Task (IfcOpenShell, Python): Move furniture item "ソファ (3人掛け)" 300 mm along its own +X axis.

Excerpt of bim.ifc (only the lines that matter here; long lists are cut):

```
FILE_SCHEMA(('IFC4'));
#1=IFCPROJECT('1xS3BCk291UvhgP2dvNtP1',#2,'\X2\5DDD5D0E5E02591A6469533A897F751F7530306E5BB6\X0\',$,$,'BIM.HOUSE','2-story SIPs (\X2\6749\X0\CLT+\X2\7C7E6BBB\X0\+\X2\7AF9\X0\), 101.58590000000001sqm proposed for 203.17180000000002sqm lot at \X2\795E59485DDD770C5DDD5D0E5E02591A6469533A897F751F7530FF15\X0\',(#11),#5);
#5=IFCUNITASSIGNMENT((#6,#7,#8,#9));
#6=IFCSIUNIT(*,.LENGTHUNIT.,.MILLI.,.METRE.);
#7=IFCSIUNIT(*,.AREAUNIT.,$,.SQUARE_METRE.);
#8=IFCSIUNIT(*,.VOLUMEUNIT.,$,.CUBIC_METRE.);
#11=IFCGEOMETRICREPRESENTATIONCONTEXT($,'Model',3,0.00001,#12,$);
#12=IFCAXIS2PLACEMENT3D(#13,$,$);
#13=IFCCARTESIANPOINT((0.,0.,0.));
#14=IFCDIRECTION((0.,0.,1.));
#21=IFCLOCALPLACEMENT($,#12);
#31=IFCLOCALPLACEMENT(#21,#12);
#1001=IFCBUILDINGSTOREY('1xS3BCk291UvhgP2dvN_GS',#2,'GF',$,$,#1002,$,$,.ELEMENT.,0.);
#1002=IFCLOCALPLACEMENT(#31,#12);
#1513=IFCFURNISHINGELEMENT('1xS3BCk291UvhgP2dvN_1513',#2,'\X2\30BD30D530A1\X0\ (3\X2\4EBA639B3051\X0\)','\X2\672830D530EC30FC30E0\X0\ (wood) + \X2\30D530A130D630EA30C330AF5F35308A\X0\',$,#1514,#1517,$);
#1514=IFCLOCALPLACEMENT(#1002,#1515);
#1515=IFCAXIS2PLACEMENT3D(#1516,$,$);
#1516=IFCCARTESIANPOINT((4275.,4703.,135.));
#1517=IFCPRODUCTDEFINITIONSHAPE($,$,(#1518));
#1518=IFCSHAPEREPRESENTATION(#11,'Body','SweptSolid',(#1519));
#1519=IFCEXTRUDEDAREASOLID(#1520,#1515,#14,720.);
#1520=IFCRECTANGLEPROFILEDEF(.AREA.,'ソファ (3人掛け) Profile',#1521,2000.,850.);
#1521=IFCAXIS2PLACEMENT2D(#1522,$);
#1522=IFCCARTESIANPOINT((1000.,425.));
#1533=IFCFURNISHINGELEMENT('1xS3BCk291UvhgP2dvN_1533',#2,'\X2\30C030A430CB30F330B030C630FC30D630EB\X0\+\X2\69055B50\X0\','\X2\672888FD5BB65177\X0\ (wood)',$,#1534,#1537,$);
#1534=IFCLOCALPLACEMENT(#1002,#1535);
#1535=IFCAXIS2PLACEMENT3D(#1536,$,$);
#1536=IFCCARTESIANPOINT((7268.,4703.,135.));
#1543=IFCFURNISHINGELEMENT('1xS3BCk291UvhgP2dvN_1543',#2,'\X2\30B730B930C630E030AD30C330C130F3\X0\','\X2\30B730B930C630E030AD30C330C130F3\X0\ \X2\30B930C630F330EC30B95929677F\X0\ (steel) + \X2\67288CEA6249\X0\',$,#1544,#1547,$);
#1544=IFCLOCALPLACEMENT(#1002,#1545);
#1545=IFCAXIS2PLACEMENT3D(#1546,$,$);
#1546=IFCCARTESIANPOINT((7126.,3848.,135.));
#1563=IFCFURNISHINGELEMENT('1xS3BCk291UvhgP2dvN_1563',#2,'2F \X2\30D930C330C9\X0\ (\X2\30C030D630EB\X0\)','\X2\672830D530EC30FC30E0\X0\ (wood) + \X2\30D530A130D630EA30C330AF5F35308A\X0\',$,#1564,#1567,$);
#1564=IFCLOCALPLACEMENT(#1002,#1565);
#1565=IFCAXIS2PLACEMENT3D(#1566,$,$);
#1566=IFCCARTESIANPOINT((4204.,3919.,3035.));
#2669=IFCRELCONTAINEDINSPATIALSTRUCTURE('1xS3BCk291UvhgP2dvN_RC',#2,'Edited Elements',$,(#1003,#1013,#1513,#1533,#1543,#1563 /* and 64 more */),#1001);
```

```python
import ifcopenshell
import ifcopenshell.api.geometry
import ifcopenshell.util.placement
import ifcopenshell.util.unit

model = ifcopenshell.open("bim.ifc")
unit_scale = ifcopenshell.util.unit.calculate_unit_scale(model)

item = model.by_guid("1xS3BCk291UvhgP2dvN_1513")
matrix = ifcopenshell.util.placement.get_local_placement(item.ObjectPlacement)
matrix[:3, 3] += matrix[:3, 0] * 0.3 / unit_scale
ifcopenshell.api.geometry.edit_object_placement(model, product=item, matrix=matrix, is_si=False)

print(ifcopenshell.util.placement.get_local_placement(item.ObjectPlacement).round(3) + 0.0)

model.write("bim_edited.ifc")
```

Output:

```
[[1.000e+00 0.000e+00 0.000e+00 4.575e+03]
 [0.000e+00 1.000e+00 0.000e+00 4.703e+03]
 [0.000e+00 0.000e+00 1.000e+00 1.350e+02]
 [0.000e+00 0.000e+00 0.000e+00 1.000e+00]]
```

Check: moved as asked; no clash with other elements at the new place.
